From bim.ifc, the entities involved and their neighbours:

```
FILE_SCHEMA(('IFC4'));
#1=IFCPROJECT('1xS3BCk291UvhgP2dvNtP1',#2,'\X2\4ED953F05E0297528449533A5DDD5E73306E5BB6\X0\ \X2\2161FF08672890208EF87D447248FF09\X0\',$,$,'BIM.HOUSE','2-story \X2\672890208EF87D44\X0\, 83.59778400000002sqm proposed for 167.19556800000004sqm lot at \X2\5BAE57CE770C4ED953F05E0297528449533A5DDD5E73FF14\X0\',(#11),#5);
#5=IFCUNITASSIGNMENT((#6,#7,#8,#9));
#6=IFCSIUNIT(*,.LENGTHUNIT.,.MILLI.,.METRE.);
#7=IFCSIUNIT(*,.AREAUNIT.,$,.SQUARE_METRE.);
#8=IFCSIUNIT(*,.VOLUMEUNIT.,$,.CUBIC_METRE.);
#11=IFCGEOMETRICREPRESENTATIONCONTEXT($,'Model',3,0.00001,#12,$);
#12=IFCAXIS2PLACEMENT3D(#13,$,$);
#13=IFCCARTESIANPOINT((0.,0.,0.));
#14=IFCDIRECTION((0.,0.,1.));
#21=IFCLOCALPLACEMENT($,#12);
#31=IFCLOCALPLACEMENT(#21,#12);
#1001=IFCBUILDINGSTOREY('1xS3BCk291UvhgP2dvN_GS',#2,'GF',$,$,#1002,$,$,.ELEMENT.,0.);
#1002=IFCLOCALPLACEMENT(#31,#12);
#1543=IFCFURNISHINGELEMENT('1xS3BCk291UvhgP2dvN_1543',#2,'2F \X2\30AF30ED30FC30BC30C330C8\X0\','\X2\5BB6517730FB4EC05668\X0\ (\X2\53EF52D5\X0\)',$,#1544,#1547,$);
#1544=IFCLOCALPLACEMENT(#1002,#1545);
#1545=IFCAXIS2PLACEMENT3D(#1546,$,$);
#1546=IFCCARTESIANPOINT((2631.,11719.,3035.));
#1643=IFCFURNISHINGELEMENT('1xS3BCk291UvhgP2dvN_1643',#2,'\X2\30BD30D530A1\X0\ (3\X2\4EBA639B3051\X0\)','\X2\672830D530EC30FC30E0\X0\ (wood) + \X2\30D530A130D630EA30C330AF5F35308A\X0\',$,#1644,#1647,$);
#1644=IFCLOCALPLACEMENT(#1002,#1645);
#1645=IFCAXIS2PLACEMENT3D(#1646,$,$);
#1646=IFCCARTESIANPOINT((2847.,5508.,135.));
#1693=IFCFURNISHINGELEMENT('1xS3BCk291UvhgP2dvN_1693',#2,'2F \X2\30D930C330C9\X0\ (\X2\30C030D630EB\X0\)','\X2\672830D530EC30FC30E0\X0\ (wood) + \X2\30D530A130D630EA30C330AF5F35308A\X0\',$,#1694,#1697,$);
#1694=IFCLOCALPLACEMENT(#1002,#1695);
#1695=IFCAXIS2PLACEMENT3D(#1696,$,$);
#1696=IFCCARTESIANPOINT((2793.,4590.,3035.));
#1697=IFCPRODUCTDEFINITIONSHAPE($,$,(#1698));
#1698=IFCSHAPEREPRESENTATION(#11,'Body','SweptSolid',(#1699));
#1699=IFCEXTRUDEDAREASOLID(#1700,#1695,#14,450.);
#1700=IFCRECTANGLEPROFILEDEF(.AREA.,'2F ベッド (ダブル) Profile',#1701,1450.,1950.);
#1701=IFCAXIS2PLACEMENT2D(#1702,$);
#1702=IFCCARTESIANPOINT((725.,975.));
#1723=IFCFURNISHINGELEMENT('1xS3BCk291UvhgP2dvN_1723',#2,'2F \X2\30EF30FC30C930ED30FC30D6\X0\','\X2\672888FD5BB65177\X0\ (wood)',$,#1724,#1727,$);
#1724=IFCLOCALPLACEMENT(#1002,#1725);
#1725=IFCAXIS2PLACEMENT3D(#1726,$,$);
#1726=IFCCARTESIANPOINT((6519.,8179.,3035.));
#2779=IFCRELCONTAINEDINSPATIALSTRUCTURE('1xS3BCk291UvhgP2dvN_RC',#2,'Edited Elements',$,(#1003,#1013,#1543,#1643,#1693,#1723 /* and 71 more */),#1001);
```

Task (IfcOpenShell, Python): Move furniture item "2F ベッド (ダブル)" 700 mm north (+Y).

```python
import ifcopenshell
import ifcopenshell.api.geometry
import ifcopenshell.util.placement

model = ifcopenshell.open("bim.ifc")

item = model.by_guid("1xS3BCk291UvhgP2dvN_1693")
matrix = ifcopenshell.util.placement.get_local_placement(item.ObjectPlacement)
matrix[1, 3] += 700.0
ifcopenshell.api.geometry.edit_object_placement(model, product=item, matrix=matrix, is_si=False)

print(ifcopenshell.util.placement.get_local_placement(item.ObjectPlacement).round(3) + 0.0)

model.write("bim-out.ifc")
```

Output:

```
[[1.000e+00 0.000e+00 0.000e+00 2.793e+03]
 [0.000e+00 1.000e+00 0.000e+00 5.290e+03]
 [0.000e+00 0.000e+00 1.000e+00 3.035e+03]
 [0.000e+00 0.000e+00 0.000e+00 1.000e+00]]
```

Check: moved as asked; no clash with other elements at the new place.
